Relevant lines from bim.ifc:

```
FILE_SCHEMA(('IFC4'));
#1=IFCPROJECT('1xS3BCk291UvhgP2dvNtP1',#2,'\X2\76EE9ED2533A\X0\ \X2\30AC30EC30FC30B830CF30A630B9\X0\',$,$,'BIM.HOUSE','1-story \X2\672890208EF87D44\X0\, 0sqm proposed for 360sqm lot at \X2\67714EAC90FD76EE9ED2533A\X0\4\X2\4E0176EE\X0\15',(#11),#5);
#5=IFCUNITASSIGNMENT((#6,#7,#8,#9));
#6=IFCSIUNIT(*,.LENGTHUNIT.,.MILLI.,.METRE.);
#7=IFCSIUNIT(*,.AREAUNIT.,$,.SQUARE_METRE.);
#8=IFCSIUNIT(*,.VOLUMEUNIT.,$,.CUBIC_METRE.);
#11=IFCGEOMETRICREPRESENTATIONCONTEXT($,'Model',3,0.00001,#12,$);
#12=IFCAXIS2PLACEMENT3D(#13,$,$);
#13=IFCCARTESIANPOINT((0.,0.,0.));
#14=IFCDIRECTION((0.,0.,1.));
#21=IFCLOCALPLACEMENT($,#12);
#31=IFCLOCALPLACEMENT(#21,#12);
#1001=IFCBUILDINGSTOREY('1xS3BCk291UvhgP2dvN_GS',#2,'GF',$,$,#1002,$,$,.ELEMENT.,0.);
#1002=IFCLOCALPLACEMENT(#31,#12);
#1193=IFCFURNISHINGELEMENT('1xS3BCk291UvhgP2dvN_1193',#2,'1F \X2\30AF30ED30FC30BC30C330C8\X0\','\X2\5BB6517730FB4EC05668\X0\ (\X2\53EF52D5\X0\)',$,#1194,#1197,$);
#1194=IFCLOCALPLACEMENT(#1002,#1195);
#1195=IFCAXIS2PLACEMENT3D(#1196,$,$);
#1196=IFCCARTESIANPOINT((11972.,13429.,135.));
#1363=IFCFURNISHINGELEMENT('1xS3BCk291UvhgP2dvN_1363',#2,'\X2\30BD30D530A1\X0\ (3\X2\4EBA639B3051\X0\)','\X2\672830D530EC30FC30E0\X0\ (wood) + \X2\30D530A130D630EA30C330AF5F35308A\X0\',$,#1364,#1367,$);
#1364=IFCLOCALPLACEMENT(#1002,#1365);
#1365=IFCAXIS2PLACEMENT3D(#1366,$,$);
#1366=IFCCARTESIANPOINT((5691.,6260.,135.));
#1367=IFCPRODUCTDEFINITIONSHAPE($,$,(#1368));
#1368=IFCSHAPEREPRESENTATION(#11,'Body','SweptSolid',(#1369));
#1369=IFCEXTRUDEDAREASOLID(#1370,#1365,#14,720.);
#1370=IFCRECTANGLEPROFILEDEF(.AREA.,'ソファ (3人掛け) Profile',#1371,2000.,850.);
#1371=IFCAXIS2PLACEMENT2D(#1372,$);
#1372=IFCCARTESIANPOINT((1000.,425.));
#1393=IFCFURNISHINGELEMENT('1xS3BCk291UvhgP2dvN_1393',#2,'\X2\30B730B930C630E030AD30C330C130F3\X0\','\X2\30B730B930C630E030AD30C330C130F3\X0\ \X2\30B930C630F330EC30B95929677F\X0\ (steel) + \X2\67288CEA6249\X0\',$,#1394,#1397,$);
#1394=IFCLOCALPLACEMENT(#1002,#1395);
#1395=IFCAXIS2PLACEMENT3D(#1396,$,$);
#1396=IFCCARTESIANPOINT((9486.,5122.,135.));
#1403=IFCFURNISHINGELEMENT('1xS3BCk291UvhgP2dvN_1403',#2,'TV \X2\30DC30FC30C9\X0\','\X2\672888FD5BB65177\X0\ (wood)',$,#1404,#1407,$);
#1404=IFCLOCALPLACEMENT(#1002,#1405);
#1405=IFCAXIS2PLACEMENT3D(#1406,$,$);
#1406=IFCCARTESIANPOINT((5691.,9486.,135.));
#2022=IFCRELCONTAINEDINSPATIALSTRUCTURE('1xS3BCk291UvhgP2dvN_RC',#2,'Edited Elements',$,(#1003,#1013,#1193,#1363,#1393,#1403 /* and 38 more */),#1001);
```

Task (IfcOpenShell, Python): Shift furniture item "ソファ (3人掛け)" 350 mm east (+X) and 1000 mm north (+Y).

```python
import ifcopenshell
import ifcopenshell.api.geometry
import ifcopenshell.util.placement
import ifcopenshell.util.unit

model = ifcopenshell.open("bim.ifc")
unit_scale = ifcopenshell.util.unit.calculate_unit_scale(model)

item = model.by_id(1363)
matrix = ifcopenshell.util.placement.get_local_placement(item.ObjectPlacement)
matrix[0, 3] += 0.35 / unit_scale
matrix[1, 3] += 1 / unit_scale
ifcopenshell.api.geometry.edit_object_placement(model, product=item, matrix=matrix, is_si=False)

print(ifcopenshell.util.placement.get_local_placement(item.ObjectPlacement).round(3) + 0.0)

model.write("bim_updated.ifc")
```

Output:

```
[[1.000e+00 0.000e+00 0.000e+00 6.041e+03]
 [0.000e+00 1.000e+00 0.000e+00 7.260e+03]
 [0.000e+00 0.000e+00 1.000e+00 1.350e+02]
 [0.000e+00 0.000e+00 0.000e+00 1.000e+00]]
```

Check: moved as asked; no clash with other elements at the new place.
